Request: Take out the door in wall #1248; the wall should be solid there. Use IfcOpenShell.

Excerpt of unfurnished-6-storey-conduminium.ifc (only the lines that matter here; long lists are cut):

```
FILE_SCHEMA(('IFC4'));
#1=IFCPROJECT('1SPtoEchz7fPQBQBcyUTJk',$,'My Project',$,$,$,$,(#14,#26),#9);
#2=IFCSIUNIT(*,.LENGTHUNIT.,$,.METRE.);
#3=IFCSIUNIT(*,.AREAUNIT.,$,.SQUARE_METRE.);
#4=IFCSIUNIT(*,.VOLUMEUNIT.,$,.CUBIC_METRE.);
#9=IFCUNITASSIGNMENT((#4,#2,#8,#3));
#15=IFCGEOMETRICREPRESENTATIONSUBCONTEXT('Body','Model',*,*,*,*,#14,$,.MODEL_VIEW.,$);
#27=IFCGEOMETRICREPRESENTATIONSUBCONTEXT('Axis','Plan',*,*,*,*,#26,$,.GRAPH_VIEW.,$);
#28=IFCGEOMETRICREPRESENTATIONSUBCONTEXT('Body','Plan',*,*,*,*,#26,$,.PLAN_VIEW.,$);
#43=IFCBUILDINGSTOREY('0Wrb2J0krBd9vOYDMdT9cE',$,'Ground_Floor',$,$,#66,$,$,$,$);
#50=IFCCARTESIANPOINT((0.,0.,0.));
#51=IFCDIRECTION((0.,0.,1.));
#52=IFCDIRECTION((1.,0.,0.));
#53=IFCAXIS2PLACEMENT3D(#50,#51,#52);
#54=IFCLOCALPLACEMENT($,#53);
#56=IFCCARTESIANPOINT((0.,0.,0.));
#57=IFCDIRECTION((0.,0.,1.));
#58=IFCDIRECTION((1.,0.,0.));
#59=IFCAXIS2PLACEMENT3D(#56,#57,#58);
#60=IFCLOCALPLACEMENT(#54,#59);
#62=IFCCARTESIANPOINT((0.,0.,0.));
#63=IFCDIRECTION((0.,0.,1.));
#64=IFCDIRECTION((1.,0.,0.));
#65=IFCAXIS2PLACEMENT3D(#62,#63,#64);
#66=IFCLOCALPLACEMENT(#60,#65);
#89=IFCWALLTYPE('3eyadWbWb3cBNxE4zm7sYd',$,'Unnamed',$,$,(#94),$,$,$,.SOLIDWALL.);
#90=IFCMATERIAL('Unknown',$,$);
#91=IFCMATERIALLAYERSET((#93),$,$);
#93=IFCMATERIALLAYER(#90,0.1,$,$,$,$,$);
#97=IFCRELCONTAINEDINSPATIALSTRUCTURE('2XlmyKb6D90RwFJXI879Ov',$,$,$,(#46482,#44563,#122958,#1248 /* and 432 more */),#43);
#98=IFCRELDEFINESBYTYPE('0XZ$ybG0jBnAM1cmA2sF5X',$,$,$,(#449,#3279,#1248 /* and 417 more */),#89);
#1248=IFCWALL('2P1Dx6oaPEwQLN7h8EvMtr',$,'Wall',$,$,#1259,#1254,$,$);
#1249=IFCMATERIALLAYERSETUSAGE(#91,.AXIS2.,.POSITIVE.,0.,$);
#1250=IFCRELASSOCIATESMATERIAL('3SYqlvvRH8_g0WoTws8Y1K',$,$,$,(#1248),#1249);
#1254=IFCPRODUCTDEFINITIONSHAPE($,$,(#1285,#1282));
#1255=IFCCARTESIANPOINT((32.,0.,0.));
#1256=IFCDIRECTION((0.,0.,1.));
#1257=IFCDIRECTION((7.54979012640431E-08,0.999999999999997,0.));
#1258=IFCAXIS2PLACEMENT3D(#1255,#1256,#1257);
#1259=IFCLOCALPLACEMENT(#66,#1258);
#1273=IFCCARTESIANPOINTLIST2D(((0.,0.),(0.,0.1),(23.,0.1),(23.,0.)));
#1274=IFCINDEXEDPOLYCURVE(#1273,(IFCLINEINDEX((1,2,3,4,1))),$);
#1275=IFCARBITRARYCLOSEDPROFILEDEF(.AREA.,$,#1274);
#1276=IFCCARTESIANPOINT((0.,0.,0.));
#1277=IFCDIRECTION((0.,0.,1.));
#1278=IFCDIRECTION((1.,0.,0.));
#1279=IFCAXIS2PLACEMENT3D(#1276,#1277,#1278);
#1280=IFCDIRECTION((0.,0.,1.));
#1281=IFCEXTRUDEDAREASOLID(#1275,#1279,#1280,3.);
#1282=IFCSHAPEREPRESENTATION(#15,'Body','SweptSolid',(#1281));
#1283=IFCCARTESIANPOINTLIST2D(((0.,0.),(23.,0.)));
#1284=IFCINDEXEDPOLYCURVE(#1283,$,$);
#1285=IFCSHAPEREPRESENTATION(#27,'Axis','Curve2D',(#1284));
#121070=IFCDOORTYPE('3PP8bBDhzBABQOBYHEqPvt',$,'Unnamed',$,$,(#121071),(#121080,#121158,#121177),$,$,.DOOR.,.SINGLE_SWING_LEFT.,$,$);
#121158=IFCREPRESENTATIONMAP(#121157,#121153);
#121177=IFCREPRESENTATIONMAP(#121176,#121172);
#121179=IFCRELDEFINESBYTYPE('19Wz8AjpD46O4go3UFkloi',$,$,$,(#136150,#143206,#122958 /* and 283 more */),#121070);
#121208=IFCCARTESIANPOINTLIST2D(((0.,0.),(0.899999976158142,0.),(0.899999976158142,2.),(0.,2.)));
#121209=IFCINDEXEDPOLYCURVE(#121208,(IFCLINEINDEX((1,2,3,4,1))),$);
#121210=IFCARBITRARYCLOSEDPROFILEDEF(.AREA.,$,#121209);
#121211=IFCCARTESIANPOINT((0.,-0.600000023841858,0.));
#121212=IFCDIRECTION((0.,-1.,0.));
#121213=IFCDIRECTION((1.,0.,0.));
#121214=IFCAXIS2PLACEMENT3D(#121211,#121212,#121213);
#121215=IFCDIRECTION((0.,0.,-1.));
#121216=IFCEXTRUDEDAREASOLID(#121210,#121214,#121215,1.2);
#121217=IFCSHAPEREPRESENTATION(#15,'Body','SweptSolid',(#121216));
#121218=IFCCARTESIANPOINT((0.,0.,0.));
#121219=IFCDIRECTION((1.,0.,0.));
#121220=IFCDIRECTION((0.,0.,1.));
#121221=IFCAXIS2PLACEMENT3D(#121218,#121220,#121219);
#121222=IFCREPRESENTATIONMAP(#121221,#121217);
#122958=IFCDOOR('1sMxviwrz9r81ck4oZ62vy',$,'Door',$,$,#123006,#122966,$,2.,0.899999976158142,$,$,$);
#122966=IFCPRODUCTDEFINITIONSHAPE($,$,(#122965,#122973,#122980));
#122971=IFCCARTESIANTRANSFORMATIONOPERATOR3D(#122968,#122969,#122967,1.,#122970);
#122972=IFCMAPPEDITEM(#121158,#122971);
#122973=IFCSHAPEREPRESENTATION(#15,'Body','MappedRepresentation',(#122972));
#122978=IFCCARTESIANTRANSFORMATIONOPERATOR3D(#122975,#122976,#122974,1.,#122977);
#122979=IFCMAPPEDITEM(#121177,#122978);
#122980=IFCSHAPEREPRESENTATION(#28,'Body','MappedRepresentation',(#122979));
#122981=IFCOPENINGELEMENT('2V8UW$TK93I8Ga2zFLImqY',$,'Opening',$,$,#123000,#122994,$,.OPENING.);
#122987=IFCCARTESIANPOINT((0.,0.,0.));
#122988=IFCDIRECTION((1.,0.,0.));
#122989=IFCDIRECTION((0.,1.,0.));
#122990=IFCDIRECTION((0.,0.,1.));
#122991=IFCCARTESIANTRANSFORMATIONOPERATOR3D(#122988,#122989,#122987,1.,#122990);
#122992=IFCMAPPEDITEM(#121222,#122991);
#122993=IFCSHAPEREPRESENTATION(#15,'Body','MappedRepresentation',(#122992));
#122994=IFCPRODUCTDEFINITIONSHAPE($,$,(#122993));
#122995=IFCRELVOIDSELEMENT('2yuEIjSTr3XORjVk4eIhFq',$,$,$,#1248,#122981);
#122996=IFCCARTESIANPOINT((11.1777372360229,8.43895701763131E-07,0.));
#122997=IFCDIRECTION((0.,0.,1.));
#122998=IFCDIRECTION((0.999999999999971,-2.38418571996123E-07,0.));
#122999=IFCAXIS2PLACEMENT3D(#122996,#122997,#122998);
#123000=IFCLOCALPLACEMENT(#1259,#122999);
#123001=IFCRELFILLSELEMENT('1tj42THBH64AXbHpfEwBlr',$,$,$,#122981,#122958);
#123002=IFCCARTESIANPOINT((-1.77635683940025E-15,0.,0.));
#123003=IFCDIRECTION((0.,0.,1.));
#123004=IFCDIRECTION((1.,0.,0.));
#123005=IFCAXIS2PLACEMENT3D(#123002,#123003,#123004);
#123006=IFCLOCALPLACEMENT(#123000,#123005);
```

```python
import ifcopenshell
import ifcopenshell.api.feature
import ifcopenshell.api.root
import ifcopenshell.geom
import ifcopenshell.util.shape

model = ifcopenshell.open("unfurnished-6-storey-conduminium.ifc")
settings = ifcopenshell.geom.settings()


def volume(element):
    """Net volume in cubic metres, openings subtracted."""
    shape = ifcopenshell.geom.create_shape(settings, element)
    return ifcopenshell.util.shape.get_volume(shape.geometry)


door = model.by_guid("1sMxviwrz9r81ck4oZ62vy")
opening = door.FillsVoids[0].RelatingOpeningElement
wall = opening.VoidsElements[0].RelatingBuildingElement
before = volume(wall)

ifcopenshell.api.root.remove_product(model, product=door)
ifcopenshell.api.feature.remove_feature(model, feature=opening)

after = volume(wall)

print(f"wall volume {before:.3f} -> {after:.3f} m3")

model.write("unfurnished-6-storey-conduminium_updated.ifc")
```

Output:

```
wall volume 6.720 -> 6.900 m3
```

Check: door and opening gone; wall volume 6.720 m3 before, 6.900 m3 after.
